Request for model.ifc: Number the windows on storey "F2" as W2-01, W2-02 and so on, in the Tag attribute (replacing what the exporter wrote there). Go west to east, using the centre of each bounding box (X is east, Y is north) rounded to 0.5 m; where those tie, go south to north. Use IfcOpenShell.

First a look at what the model holds.

```python
import ifcopenshell
import ifcopenshell.util.element
import ifcopenshell.util.placement

model = ifcopenshell.open("model.ifc")
print(model.schema)
storey = next(s for s in model.by_type("IfcBuildingStorey") if s.Name == "F2")
windows = [e for e in ifcopenshell.util.element.get_decomposition(storey) if e.is_a("IfcWindow")]
for e in sorted(windows, key=lambda e: e.id()):
    origin = ifcopenshell.util.placement.get_local_placement(e.ObjectPlacement)[:3, 3]
    print(e.id(), e.Tag, e.Name, origin.round(2) + 0.0, sep=" | ")
```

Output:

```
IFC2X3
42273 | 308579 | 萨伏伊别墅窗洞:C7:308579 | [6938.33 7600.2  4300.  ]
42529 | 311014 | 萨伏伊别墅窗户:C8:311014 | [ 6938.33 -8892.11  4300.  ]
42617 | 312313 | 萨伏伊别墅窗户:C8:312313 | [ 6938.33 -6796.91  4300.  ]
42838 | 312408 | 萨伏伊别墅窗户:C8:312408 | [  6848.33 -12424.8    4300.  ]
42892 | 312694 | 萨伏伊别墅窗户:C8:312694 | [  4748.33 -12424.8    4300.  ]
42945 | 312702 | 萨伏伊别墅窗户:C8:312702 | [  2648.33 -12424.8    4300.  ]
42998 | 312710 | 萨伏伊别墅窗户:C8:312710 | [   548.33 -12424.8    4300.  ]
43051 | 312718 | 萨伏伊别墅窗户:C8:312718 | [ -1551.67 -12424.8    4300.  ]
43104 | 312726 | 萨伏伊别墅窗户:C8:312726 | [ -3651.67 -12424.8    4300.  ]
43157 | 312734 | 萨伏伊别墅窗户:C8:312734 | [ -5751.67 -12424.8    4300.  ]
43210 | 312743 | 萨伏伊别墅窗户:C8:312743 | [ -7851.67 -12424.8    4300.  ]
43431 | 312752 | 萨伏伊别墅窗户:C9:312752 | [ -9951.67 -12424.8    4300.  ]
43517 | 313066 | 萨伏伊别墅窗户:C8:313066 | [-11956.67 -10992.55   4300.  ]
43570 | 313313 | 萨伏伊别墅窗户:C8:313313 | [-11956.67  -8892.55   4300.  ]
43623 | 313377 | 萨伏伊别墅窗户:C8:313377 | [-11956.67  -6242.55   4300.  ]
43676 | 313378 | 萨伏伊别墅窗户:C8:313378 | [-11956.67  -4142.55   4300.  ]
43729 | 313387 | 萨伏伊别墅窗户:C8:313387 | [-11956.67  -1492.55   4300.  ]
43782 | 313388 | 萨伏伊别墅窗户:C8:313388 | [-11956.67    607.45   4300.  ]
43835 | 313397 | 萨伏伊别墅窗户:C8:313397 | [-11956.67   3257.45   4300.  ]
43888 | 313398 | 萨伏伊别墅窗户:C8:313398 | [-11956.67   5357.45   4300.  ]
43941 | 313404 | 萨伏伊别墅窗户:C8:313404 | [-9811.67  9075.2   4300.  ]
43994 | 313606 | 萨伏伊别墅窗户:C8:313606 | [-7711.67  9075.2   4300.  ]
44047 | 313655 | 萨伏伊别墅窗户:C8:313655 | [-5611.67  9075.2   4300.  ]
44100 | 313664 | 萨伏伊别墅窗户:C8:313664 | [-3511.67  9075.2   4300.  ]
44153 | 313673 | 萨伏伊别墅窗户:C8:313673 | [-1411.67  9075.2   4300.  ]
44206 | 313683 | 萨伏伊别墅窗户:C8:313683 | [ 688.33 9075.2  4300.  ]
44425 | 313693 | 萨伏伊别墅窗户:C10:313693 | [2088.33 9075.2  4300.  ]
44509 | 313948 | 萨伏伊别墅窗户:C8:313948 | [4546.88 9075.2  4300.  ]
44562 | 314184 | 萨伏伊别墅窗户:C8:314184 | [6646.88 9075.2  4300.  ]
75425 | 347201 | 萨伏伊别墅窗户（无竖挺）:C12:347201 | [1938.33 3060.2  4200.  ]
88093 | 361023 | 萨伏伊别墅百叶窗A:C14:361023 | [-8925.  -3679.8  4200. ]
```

```python
import ifcopenshell
import ifcopenshell.geom
import ifcopenshell.util.element
import ifcopenshell.util.shape

model = ifcopenshell.open("model.ifc")
settings = ifcopenshell.geom.settings()
settings.set("use-world-coords", True)


def centre(element):
    shape = ifcopenshell.geom.create_shape(settings, element)
    return ifcopenshell.util.shape.get_bbox_centroid(shape.geometry)


storey = next(s for s in model.by_type("IfcBuildingStorey") if s.Name == "F2")
windows = [e for e in ifcopenshell.util.element.get_decomposition(storey) if e.is_a("IfcWindow")]

# Insertion points can sit at a corner or the storey origin, so sort by the geometry (in metres).
centres = {e: centre(e) for e in windows}
windows.sort(key=lambda e: (round(centres[e][0] / 0.5), centres[e][1]))

for i, e in enumerate(windows, start=1):
    number = f"W2-{i:02d}"
    e.Tag = number
    print(e.id(), number)

model.write("model_v2.ifc")
```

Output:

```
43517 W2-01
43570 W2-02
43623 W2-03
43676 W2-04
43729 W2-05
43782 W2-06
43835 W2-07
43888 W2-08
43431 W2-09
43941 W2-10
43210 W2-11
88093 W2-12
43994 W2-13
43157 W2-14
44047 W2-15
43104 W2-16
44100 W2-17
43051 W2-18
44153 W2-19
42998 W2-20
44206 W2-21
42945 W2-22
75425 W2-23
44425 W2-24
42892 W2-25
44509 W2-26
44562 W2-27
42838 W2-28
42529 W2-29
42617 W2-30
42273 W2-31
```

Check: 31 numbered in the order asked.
